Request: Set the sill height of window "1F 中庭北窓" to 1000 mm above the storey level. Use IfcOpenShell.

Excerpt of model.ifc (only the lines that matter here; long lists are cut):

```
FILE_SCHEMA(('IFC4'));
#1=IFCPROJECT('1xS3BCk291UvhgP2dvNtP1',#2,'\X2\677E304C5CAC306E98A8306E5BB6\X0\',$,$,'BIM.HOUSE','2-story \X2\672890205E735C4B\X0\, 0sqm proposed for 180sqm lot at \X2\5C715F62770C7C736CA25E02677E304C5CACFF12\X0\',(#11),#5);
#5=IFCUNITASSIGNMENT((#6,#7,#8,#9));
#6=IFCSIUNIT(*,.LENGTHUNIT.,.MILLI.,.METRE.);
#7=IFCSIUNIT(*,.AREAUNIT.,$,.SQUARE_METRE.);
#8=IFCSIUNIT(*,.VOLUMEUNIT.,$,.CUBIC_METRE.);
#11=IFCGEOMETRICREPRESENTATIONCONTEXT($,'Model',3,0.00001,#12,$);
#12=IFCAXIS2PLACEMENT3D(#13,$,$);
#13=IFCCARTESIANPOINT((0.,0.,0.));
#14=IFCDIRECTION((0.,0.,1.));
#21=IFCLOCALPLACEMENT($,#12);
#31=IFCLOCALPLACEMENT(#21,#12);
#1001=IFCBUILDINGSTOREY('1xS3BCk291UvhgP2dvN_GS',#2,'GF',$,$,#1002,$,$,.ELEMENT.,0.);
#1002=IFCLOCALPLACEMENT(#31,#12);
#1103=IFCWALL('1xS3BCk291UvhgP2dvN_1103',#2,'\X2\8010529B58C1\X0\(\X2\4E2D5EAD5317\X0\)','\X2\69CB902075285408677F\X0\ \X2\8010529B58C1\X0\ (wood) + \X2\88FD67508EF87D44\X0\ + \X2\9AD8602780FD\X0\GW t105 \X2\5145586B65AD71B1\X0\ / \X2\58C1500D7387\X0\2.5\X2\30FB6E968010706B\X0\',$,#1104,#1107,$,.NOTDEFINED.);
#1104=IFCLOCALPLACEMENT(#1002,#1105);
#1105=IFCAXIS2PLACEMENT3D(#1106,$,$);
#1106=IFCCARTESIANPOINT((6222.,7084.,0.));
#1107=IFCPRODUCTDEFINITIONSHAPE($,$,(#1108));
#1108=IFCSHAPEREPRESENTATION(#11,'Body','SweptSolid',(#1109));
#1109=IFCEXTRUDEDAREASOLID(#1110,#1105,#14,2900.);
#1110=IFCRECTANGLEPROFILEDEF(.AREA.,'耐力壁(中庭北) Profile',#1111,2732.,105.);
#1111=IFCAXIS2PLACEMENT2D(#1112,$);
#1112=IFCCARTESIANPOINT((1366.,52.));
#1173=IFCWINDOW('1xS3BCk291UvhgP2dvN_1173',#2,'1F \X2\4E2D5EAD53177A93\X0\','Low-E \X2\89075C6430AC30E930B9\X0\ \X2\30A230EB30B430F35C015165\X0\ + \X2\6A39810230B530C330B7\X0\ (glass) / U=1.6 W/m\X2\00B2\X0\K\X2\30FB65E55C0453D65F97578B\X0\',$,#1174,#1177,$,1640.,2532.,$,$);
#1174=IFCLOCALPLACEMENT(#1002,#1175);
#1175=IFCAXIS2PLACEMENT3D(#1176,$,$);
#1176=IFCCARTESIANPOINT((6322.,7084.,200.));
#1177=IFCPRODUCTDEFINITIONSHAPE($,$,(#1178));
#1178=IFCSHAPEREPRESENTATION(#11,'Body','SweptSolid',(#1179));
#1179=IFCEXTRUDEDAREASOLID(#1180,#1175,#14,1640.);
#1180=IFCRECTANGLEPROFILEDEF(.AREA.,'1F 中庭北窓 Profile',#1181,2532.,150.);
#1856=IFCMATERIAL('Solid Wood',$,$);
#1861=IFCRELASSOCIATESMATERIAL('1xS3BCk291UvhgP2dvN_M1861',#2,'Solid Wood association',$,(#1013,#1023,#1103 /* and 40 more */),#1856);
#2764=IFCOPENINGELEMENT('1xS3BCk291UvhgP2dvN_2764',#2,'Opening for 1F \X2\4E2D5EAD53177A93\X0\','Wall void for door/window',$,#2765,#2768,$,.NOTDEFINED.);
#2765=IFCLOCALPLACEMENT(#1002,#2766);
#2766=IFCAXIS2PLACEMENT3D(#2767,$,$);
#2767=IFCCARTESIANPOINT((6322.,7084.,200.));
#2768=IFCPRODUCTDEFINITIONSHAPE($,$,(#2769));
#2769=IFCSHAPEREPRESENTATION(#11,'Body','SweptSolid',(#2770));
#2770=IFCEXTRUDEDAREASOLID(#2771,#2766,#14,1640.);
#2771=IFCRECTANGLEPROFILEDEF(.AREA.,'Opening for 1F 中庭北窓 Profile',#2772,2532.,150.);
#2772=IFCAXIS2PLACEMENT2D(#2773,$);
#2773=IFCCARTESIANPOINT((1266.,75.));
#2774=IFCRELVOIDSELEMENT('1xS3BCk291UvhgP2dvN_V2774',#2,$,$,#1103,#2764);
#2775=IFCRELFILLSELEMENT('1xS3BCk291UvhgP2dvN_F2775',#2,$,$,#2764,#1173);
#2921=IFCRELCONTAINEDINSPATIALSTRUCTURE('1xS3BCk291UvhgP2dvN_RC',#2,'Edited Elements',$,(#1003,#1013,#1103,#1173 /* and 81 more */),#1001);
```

```python
import numpy as np
import ifcopenshell
import ifcopenshell.api.geometry
import ifcopenshell.geom
import ifcopenshell.util.element
import ifcopenshell.util.placement
import ifcopenshell.util.shape
import ifcopenshell.util.unit

model = ifcopenshell.open("model.ifc")
unit_scale = ifcopenshell.util.unit.calculate_unit_scale(model)

window = model.by_guid("1xS3BCk291UvhgP2dvN_1173")
opening = window.FillsVoids[0].RelatingOpeningElement
storey = ifcopenshell.util.element.get_container(window, ifc_class="IfcBuildingStorey")
level = ifcopenshell.util.placement.get_local_placement(storey.ObjectPlacement)[2, 3]

# The opening's origin need not be at the sill, so measure its lowest point.
shape = ifcopenshell.geom.create_shape(ifcopenshell.geom.settings(), opening)
bottom = ifcopenshell.util.shape.get_shape_bottom_elevation(shape, shape.geometry) / unit_scale
dz = level + 1 / unit_scale - bottom

shift = np.array([0.0, 0.0, dz])
# The window is not placed relative to its opening, so move both.
for product in (opening, window):
    matrix = ifcopenshell.util.placement.get_local_placement(product.ObjectPlacement)
    matrix[:3, 3] += shift
    ifcopenshell.api.geometry.edit_object_placement(model, product=product, matrix=matrix, is_si=False)

print(f"moved by {dz * unit_scale:+.3f} m")

model.write("model_updated.ifc")
```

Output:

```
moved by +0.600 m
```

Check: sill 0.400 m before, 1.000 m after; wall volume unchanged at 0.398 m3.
